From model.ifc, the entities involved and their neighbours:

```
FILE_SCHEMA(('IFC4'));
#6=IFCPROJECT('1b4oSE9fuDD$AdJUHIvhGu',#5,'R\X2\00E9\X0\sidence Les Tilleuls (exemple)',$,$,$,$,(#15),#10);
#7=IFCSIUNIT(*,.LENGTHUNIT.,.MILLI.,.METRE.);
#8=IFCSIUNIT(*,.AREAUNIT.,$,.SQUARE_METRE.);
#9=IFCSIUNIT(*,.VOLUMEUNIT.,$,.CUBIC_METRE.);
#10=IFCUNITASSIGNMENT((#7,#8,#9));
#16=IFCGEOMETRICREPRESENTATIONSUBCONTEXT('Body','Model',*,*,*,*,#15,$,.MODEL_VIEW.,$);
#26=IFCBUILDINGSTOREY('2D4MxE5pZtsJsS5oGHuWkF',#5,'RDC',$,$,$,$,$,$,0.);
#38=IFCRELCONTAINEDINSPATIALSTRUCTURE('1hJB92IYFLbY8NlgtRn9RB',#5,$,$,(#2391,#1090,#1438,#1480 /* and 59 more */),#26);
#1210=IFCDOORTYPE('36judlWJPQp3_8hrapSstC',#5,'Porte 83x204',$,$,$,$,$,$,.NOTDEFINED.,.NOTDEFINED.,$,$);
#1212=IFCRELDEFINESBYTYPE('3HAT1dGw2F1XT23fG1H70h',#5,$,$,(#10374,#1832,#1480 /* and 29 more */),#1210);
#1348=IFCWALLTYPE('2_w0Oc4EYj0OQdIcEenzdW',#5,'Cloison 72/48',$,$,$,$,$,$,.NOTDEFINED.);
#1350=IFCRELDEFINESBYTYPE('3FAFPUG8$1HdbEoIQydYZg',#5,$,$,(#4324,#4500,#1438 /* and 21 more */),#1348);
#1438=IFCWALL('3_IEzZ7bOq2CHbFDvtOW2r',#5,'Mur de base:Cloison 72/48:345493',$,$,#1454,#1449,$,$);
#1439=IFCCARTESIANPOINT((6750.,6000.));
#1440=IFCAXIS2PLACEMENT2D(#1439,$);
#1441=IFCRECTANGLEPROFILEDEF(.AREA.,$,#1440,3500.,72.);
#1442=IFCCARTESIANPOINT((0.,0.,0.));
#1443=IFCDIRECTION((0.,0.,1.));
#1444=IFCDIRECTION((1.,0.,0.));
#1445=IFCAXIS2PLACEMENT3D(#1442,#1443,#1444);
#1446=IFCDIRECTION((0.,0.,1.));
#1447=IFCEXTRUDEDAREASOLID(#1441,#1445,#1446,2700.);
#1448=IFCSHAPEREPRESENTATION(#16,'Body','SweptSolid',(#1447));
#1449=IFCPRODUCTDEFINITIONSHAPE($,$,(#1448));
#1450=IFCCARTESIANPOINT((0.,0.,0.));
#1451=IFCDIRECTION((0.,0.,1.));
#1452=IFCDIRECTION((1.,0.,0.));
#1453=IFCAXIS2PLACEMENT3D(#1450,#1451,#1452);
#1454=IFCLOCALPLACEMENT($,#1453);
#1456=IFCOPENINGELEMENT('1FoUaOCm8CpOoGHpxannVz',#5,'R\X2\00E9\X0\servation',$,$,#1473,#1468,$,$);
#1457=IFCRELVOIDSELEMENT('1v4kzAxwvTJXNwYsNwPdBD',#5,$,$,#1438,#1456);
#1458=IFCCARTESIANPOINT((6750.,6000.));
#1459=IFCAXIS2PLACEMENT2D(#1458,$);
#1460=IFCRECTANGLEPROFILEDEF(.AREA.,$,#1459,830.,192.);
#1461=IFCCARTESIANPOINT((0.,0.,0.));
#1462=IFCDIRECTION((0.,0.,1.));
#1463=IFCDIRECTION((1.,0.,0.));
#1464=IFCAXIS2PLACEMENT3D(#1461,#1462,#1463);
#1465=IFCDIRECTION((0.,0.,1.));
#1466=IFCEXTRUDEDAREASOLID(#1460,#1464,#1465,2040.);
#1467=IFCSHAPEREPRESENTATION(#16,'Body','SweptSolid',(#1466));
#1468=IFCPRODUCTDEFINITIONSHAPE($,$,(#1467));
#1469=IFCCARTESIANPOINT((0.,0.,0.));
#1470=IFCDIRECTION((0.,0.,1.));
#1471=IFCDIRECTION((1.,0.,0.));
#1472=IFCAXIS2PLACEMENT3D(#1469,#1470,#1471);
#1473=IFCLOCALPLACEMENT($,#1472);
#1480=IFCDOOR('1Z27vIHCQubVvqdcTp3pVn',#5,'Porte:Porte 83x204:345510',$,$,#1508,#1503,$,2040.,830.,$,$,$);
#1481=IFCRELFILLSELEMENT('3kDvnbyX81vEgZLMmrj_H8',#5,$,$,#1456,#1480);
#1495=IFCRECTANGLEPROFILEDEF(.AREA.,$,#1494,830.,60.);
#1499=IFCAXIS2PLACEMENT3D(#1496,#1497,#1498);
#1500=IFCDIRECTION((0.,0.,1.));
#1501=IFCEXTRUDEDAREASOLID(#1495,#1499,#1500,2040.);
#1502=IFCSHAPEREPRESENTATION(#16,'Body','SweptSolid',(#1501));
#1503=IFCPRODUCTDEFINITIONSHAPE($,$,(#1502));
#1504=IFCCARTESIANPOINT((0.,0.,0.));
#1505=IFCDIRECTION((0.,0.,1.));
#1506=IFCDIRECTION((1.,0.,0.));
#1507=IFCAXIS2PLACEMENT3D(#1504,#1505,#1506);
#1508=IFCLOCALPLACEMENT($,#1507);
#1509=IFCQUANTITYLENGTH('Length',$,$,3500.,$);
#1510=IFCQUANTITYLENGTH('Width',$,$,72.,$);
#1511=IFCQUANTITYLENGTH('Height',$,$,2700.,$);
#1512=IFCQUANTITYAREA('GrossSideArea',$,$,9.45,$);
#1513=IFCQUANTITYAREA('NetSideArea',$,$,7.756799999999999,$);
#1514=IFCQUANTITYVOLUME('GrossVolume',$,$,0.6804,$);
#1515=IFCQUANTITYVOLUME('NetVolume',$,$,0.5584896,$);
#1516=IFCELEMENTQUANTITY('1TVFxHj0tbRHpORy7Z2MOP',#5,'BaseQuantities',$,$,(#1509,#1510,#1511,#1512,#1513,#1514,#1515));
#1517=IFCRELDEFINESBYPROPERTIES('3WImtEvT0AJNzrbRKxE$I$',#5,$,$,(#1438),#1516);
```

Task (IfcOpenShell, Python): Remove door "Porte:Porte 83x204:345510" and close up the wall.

```python
import ifcopenshell
import ifcopenshell.api.feature
import ifcopenshell.api.pset
import ifcopenshell.api.root
import ifcopenshell.geom
import ifcopenshell.util.element
import ifcopenshell.util.shape
import ifcopenshell.util.unit

model = ifcopenshell.open("model.ifc")
area_scale = ifcopenshell.util.unit.calculate_unit_scale(model, "AREAUNIT")
volume_scale = ifcopenshell.util.unit.calculate_unit_scale(model, "VOLUMEUNIT")
settings = ifcopenshell.geom.settings()


def volume(element):
    """Net volume in cubic metres, openings subtracted."""
    shape = ifcopenshell.geom.create_shape(settings, element)
    return ifcopenshell.util.shape.get_volume(shape.geometry)


door = model.by_guid("1Z27vIHCQubVvqdcTp3pVn")
opening = door.FillsVoids[0].RelatingOpeningElement
wall = opening.VoidsElements[0].RelatingBuildingElement
before = volume(wall)

ifcopenshell.api.root.remove_product(model, product=door)
ifcopenshell.api.feature.remove_feature(model, feature=opening)

after = volume(wall)
thickness = 0.072  # wall thickness in metres

# Update the wall's stored quantities.
qto = model.by_id(ifcopenshell.util.element.get_pset(wall, "BaseQuantities", should_inherit=False)["id"])
ifcopenshell.api.pset.edit_qto(model, qto=qto, properties={
    "NetSideArea": after / thickness / area_scale,
    "NetVolume": after / volume_scale,
})

print(f"wall volume {before:.3f} -> {after:.3f} m3")

model.write("model_edited.ifc")
```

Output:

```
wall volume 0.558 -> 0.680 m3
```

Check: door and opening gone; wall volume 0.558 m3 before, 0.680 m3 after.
